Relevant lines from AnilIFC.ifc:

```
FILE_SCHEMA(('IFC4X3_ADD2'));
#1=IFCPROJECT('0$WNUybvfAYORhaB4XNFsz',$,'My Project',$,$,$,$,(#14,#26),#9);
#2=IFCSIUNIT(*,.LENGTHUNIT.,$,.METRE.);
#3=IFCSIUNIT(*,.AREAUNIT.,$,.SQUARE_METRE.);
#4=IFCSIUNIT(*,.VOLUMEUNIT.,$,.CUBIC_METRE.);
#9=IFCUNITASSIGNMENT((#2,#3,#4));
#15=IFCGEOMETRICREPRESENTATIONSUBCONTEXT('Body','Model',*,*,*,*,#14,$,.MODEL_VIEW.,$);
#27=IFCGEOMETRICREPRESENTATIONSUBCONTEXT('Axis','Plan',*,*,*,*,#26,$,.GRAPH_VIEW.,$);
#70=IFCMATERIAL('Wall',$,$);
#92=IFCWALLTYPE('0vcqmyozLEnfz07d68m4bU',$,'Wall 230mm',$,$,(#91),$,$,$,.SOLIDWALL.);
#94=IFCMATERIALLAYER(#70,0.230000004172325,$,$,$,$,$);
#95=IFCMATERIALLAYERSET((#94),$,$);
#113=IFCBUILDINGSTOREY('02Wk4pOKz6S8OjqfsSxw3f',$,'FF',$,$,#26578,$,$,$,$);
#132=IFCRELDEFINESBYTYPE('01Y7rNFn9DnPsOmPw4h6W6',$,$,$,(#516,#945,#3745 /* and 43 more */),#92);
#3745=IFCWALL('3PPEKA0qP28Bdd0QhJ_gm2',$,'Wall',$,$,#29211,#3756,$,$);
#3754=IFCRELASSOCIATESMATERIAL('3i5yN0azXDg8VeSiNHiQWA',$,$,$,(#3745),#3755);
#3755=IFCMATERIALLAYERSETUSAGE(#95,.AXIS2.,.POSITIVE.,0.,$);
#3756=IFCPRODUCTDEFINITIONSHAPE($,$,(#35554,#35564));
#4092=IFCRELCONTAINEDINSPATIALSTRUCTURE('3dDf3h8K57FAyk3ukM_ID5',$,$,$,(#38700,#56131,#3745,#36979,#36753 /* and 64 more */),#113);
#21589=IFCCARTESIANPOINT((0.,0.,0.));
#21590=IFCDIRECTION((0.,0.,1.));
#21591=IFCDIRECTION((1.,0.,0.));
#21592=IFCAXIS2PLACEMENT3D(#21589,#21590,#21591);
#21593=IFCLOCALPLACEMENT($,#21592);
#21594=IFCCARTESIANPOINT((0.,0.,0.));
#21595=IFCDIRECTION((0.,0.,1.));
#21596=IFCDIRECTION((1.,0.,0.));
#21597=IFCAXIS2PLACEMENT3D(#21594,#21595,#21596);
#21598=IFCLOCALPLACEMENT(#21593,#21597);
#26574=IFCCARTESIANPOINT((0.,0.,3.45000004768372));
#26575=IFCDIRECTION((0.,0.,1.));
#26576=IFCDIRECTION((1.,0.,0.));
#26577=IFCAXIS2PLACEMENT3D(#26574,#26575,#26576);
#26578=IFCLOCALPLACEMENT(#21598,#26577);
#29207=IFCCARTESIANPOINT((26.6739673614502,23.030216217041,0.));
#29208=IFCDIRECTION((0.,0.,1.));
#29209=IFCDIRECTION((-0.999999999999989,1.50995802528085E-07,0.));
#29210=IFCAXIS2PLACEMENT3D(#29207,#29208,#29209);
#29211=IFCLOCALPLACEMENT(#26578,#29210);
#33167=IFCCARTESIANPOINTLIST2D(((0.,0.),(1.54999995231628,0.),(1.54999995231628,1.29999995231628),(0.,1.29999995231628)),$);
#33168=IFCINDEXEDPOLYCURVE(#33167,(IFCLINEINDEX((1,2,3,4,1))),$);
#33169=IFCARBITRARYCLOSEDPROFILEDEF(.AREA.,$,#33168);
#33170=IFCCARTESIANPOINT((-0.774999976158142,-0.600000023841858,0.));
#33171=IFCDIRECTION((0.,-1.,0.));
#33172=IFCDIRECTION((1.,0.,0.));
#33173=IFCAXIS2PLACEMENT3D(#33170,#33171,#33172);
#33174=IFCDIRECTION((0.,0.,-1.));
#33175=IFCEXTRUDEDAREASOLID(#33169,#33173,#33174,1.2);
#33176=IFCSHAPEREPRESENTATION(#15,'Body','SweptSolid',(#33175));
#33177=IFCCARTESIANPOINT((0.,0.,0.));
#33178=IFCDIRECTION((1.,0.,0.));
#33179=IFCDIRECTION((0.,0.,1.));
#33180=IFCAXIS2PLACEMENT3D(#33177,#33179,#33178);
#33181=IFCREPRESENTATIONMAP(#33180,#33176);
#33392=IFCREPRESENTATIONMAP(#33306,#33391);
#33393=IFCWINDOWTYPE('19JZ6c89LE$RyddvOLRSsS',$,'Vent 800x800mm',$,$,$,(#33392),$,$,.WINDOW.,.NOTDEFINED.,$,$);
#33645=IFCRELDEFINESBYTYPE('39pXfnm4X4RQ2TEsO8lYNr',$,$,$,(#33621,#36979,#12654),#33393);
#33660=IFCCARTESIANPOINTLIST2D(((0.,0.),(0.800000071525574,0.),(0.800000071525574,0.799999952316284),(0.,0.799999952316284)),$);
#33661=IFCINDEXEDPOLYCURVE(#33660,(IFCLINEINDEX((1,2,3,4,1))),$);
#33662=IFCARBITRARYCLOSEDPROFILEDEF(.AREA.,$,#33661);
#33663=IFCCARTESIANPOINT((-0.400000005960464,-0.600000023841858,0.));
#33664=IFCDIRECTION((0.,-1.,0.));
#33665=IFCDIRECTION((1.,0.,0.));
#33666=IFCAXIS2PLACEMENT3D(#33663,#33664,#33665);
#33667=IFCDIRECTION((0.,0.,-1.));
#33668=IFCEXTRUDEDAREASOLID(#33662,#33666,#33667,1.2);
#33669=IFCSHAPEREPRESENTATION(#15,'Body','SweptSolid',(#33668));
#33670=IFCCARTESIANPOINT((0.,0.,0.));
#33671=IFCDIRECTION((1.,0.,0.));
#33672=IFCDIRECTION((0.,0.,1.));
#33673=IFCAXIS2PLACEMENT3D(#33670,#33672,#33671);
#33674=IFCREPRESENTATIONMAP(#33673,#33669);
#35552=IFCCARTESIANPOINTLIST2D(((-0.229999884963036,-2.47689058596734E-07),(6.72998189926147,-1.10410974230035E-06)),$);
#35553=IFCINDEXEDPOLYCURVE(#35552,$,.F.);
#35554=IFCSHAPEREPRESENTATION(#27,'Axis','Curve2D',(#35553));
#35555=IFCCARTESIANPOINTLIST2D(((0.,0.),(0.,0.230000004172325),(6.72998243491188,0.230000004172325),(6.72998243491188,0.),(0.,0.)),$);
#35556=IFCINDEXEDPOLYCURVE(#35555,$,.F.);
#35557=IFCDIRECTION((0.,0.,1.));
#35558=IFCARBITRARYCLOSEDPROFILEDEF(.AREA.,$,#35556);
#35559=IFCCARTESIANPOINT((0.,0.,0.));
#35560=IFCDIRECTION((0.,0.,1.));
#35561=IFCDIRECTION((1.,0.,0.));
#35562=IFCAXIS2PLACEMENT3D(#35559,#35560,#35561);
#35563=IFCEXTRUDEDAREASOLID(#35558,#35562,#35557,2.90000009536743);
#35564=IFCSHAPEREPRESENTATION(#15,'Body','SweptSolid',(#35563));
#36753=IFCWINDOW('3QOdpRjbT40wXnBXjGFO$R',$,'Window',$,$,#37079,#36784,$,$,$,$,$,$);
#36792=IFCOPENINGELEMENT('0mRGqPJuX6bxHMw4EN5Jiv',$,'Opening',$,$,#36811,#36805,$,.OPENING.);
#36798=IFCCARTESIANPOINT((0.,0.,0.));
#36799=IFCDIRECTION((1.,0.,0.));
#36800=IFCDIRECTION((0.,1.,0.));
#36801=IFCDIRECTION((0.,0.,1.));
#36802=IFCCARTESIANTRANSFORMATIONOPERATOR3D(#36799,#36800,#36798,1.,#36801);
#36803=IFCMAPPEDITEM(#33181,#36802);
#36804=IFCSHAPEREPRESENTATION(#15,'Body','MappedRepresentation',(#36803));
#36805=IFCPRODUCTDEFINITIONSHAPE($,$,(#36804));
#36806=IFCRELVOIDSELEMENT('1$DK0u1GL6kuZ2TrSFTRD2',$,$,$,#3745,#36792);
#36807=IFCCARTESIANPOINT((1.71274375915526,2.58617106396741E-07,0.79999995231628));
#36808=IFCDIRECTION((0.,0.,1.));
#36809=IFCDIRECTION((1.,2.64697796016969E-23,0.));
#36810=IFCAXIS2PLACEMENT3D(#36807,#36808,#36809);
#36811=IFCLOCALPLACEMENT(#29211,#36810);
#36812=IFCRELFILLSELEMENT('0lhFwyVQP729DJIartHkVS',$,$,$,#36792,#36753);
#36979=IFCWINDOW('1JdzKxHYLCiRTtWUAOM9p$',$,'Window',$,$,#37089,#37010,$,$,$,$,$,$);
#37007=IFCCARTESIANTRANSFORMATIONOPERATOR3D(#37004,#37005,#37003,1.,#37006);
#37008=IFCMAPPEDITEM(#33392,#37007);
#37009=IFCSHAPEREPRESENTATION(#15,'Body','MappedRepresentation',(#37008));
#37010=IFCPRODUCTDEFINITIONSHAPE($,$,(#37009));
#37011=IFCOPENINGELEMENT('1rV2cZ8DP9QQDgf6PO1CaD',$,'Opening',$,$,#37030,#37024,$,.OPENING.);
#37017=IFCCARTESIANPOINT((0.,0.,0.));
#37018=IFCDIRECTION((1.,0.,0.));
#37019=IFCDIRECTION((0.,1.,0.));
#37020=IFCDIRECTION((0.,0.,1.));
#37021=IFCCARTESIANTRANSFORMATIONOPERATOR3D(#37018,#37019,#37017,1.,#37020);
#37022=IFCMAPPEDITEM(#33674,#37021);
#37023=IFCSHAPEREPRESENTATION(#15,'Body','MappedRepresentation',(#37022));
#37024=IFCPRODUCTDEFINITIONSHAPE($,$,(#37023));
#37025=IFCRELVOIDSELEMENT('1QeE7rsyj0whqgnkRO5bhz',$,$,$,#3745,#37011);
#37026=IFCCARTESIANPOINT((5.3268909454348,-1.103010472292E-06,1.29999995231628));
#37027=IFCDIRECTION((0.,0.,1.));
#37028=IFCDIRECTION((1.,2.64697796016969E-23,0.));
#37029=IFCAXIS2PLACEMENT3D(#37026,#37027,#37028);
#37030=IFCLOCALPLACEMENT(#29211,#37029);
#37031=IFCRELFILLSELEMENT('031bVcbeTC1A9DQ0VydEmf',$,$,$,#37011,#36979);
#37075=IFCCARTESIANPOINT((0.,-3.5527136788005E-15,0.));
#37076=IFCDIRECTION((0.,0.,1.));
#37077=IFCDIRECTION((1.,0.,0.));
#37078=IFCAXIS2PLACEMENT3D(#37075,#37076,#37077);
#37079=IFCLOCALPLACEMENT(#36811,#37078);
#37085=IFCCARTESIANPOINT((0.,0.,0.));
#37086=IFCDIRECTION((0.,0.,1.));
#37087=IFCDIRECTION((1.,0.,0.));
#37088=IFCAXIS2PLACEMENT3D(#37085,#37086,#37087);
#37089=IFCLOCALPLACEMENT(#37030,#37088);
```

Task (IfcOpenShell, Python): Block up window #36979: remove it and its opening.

```python
import ifcopenshell
import ifcopenshell.api.feature
import ifcopenshell.api.root
import ifcopenshell.geom
import ifcopenshell.util.shape

model = ifcopenshell.open("AnilIFC.ifc")
settings = ifcopenshell.geom.settings()


def volume(element):
    """Net volume in cubic metres, openings subtracted."""
    shape = ifcopenshell.geom.create_shape(settings, element)
    return ifcopenshell.util.shape.get_volume(shape.geometry)


window = model.by_guid("1JdzKxHYLCiRTtWUAOM9p$")
opening = window.FillsVoids[0].RelatingOpeningElement
wall = opening.VoidsElements[0].RelatingBuildingElement
before = volume(wall)

ifcopenshell.api.root.remove_product(model, product=window)
ifcopenshell.api.feature.remove_feature(model, feature=opening)

after = volume(wall)

print(f"wall volume {before:.3f} -> {after:.3f} m3")

model.write("AnilIFC_rev.ifc")
```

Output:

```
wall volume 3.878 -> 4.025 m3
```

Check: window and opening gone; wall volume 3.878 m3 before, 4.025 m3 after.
